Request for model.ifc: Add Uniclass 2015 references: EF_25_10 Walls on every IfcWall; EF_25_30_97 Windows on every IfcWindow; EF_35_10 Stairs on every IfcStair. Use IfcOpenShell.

First a look at what the model holds.

```python
import ifcopenshell

model = ifcopenshell.open("model.ifc")
print(model.schema)
print("classifications:", [c.Name for c in model.by_type("IfcClassification")])
for ifc_class in ("IfcDoor", "IfcRoof", "IfcStair", "IfcWall", "IfcWindow"):
    print(ifc_class, len(model.by_type(ifc_class)))
```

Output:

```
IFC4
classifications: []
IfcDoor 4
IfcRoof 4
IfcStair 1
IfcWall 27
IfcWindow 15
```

```python
import ifcopenshell
import ifcopenshell.api.classification

model = ifcopenshell.open("model.ifc")

system = ifcopenshell.api.classification.add_classification(model, classification="Uniclass 2015")

codes = {
    "IfcWall": ("EF_25_10", "Walls"),
    "IfcWindow": ("EF_25_30_97", "Windows"),
    "IfcStair": ("EF_35_10", "Stairs"),
}
for ifc_class, (code, name) in codes.items():
    products = model.by_type(ifc_class)
    ifcopenshell.api.classification.add_reference(
        model, products=products, classification=system, identification=code, name=name
    )
    print(code, len(products))

model.write("model_v2.ifc")
```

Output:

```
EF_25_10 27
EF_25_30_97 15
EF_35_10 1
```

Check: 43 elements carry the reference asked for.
